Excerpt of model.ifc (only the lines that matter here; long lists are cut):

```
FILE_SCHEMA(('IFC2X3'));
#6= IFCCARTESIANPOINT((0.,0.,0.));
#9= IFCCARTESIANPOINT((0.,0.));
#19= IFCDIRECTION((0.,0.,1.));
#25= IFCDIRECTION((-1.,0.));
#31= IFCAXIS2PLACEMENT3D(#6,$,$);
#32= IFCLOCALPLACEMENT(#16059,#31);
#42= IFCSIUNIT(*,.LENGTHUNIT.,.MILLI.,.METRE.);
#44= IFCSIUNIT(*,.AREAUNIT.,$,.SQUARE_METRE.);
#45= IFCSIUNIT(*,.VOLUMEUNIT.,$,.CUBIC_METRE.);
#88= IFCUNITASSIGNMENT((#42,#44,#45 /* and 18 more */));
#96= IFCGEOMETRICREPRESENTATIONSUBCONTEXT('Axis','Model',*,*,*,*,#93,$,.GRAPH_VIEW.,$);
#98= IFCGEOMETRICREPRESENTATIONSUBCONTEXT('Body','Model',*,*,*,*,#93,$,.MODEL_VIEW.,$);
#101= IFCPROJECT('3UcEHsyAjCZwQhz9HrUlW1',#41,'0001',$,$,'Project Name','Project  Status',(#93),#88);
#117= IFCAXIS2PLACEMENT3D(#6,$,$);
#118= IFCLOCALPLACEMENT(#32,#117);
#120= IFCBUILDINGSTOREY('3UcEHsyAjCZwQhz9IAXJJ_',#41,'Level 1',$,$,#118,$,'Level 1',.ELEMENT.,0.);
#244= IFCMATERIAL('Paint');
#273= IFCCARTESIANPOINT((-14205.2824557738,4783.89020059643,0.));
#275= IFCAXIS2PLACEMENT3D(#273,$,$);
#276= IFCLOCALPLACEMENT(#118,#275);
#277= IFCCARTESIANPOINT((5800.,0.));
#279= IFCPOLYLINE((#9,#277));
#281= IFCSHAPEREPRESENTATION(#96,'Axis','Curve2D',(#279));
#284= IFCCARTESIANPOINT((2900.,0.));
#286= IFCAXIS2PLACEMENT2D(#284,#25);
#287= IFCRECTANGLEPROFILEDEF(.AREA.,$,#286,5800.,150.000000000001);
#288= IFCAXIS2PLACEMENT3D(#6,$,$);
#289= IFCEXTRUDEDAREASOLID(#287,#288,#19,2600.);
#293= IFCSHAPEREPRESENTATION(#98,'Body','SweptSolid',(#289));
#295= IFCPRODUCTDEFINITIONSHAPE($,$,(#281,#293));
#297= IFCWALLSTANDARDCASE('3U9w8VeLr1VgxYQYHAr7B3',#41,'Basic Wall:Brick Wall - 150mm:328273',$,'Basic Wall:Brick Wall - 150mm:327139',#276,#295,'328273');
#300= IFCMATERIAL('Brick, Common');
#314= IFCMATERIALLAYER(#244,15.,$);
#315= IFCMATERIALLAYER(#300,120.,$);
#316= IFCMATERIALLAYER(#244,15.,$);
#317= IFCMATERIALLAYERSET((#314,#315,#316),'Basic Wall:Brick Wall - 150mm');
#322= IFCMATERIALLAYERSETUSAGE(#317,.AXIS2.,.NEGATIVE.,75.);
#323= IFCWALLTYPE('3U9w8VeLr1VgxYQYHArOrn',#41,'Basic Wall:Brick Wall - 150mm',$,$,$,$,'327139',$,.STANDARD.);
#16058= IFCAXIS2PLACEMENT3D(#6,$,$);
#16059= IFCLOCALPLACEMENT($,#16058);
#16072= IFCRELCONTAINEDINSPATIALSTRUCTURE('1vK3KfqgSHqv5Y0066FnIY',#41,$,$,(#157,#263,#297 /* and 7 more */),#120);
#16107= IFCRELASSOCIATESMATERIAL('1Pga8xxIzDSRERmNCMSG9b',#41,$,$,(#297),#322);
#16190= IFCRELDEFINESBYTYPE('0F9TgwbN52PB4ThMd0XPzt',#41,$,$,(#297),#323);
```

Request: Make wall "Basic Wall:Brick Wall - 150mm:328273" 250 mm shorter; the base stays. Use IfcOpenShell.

```python
import ifcopenshell
import ifcopenshell.geom
import ifcopenshell.util.representation
import ifcopenshell.util.shape
import ifcopenshell.util.unit

model = ifcopenshell.open("model.ifc")
unit_scale = ifcopenshell.util.unit.calculate_unit_scale(model)
settings = ifcopenshell.geom.settings()


def volume(element):
    """Net volume in cubic metres, openings subtracted."""
    shape = ifcopenshell.geom.create_shape(settings, element)
    return ifcopenshell.util.shape.get_volume(shape.geometry)


wall = model.by_guid("3U9w8VeLr1VgxYQYHAr7B3")
before = volume(wall)

body = ifcopenshell.util.representation.get_representation(wall, "Model", "Body")
solid = body.Items[0]
old_height = solid.Depth
solid.Depth -= 0.25 / unit_scale
after = volume(wall)

print(f"height {old_height:g} -> {solid.Depth:g}, volume {before:.3f} -> {after:.3f} m3")

model.write("model_updated.ifc")
```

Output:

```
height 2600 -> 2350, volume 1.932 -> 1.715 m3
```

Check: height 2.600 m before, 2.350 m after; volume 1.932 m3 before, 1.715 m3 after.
